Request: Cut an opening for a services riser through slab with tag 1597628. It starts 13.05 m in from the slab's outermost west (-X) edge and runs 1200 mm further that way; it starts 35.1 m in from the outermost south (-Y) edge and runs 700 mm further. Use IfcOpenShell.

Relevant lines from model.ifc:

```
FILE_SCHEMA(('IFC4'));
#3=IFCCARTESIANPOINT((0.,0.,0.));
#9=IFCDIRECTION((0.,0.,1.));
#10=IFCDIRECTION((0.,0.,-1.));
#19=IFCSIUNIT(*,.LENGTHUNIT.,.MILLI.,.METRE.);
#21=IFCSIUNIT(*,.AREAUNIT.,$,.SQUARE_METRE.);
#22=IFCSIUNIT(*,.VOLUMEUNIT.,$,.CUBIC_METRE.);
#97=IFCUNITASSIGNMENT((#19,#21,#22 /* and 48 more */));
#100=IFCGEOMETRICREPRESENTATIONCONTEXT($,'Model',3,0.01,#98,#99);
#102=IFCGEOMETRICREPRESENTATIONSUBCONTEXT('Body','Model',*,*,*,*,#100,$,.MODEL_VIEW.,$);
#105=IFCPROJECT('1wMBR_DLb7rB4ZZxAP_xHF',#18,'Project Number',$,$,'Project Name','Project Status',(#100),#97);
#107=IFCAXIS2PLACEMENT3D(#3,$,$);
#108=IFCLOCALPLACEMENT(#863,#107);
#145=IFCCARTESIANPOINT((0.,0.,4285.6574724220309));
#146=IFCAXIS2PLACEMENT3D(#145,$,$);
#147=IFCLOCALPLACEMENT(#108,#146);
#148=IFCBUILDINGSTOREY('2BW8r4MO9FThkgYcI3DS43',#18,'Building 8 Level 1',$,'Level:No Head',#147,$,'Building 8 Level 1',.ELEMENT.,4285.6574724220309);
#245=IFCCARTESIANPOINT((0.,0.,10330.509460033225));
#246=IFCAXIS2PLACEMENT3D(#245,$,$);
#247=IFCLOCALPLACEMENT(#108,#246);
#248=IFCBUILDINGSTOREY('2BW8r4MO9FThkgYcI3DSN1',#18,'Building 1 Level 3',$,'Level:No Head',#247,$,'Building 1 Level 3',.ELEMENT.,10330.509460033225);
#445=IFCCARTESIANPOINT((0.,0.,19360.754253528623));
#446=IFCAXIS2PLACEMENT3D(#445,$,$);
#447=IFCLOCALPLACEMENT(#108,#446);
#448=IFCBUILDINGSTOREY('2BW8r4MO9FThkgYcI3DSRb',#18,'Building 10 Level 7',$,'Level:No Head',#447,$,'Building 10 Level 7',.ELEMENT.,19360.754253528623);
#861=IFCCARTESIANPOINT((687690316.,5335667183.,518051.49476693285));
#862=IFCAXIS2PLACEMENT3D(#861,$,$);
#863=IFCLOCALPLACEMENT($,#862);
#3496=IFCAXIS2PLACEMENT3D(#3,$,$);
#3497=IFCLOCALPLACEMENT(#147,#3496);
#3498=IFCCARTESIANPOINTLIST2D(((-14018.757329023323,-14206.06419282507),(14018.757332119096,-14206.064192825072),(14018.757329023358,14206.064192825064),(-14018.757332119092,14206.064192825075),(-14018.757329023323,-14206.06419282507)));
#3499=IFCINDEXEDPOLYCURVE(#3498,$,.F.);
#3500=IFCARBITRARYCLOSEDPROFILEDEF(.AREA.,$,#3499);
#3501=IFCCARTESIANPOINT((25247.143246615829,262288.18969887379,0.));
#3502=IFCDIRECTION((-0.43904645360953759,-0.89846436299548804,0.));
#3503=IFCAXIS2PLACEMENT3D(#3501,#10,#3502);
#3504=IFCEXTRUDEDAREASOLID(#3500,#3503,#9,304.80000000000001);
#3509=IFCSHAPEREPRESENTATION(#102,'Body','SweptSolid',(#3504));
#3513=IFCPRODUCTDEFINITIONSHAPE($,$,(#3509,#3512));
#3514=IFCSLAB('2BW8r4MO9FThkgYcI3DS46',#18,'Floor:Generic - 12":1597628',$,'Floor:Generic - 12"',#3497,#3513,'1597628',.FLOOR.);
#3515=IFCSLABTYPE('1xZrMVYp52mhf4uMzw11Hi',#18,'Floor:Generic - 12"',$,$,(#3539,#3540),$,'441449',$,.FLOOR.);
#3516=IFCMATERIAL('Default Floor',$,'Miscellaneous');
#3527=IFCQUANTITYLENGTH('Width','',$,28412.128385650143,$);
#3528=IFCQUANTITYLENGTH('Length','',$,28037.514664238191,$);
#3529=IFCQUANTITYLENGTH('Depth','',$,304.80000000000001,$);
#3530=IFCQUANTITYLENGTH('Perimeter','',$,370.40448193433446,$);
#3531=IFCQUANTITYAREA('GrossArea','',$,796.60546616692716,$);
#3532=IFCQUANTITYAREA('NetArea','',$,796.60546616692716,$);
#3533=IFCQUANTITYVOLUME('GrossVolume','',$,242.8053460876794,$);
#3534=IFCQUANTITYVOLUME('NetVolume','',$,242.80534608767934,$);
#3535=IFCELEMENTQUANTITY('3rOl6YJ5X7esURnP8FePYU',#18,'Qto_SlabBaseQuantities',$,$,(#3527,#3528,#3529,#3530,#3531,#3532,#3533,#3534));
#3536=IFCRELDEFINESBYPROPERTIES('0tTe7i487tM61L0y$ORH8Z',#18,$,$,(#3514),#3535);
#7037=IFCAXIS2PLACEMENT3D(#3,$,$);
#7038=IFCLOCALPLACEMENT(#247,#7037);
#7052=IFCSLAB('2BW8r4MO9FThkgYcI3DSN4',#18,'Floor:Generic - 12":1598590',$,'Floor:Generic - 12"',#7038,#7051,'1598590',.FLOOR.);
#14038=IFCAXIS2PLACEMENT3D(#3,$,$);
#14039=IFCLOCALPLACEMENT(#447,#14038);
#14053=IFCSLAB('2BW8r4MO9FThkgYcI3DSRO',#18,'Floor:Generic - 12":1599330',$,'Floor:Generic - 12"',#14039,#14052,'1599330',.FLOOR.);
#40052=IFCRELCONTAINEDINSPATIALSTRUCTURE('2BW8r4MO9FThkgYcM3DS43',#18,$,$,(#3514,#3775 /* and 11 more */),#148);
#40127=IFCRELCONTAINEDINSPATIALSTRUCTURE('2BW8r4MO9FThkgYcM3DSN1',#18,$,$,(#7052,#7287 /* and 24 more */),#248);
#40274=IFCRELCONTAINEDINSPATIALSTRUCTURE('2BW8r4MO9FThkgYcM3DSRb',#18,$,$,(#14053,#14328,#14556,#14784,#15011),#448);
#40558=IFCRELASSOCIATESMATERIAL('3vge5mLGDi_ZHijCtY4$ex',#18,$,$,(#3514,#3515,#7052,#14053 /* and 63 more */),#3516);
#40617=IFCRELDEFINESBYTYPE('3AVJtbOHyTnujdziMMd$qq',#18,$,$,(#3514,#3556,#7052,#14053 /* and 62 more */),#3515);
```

```python
import numpy as np
import ifcopenshell
import ifcopenshell.api.feature
import ifcopenshell.api.geometry
import ifcopenshell.api.pset
import ifcopenshell.api.root
import ifcopenshell.geom
import ifcopenshell.util.element
import ifcopenshell.util.placement
import ifcopenshell.util.representation
import ifcopenshell.util.shape
import ifcopenshell.util.unit

model = ifcopenshell.open("model.ifc")
unit_scale = ifcopenshell.util.unit.calculate_unit_scale(model)
area_scale = ifcopenshell.util.unit.calculate_unit_scale(model, "AREAUNIT")
volume_scale = ifcopenshell.util.unit.calculate_unit_scale(model, "VOLUMEUNIT")
settings = ifcopenshell.geom.settings()


def volume(element):
    """Net volume in cubic metres, openings subtracted."""
    shape = ifcopenshell.geom.create_shape(settings, element)
    return ifcopenshell.util.shape.get_volume(shape.geometry)


slab = model.by_guid("2BW8r4MO9FThkgYcI3DS46")
before = volume(slab)

# Extent in the slab's own axes, in metres. The edges named are its -X and -Y sides.
slab_shape = ifcopenshell.geom.create_shape(settings, slab)
vertices = ifcopenshell.util.shape.get_vertices(slab_shape.geometry)
x_min, y_min, bottom = vertices.min(axis=0)
top = vertices[:, 2].max()

opening = ifcopenshell.api.root.create_entity(model, ifc_class="IfcOpeningElement", name="Services riser opening", predefined_type="OPENING")
context = ifcopenshell.util.representation.get_context(model, "Model", "Body", "MODEL_VIEW")
width, depth = 1.2, 0.7
outline = [(0.0, 0.0), (width, 0.0), (width, depth), (0.0, depth), (0.0, 0.0)]
# Overshoot both faces by 50 mm so the cut is clean.
shape = ifcopenshell.api.geometry.add_slab_representation(
    model, context=context, depth=top - bottom + 0.1, polyline=outline
)
ifcopenshell.api.geometry.assign_representation(model, product=opening, representation=shape)

matrix = ifcopenshell.util.placement.get_local_placement(slab.ObjectPlacement)
matrix[:, 3] = matrix @ np.append(np.array([x_min + 13.05, y_min + 35.1, bottom - 0.05]) / unit_scale, 1.0)
ifcopenshell.api.geometry.edit_object_placement(model, product=opening, matrix=matrix, is_si=False)
ifcopenshell.api.feature.add_feature(model, feature=opening, element=slab)

after = volume(slab)

# Update the slab's stored quantities.
qto = model.by_id(ifcopenshell.util.element.get_pset(slab, "Qto_SlabBaseQuantities", should_inherit=False)["id"])
ifcopenshell.api.pset.edit_qto(model, qto=qto, properties={
    "NetArea": after / (top - bottom) / area_scale,
    "NetVolume": after / volume_scale,
})

print(f"slab volume {before:.3f} -> {after:.3f} m3")

model.write("model_edited.ifc")
```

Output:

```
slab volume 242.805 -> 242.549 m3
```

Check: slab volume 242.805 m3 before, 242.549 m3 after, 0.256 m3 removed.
